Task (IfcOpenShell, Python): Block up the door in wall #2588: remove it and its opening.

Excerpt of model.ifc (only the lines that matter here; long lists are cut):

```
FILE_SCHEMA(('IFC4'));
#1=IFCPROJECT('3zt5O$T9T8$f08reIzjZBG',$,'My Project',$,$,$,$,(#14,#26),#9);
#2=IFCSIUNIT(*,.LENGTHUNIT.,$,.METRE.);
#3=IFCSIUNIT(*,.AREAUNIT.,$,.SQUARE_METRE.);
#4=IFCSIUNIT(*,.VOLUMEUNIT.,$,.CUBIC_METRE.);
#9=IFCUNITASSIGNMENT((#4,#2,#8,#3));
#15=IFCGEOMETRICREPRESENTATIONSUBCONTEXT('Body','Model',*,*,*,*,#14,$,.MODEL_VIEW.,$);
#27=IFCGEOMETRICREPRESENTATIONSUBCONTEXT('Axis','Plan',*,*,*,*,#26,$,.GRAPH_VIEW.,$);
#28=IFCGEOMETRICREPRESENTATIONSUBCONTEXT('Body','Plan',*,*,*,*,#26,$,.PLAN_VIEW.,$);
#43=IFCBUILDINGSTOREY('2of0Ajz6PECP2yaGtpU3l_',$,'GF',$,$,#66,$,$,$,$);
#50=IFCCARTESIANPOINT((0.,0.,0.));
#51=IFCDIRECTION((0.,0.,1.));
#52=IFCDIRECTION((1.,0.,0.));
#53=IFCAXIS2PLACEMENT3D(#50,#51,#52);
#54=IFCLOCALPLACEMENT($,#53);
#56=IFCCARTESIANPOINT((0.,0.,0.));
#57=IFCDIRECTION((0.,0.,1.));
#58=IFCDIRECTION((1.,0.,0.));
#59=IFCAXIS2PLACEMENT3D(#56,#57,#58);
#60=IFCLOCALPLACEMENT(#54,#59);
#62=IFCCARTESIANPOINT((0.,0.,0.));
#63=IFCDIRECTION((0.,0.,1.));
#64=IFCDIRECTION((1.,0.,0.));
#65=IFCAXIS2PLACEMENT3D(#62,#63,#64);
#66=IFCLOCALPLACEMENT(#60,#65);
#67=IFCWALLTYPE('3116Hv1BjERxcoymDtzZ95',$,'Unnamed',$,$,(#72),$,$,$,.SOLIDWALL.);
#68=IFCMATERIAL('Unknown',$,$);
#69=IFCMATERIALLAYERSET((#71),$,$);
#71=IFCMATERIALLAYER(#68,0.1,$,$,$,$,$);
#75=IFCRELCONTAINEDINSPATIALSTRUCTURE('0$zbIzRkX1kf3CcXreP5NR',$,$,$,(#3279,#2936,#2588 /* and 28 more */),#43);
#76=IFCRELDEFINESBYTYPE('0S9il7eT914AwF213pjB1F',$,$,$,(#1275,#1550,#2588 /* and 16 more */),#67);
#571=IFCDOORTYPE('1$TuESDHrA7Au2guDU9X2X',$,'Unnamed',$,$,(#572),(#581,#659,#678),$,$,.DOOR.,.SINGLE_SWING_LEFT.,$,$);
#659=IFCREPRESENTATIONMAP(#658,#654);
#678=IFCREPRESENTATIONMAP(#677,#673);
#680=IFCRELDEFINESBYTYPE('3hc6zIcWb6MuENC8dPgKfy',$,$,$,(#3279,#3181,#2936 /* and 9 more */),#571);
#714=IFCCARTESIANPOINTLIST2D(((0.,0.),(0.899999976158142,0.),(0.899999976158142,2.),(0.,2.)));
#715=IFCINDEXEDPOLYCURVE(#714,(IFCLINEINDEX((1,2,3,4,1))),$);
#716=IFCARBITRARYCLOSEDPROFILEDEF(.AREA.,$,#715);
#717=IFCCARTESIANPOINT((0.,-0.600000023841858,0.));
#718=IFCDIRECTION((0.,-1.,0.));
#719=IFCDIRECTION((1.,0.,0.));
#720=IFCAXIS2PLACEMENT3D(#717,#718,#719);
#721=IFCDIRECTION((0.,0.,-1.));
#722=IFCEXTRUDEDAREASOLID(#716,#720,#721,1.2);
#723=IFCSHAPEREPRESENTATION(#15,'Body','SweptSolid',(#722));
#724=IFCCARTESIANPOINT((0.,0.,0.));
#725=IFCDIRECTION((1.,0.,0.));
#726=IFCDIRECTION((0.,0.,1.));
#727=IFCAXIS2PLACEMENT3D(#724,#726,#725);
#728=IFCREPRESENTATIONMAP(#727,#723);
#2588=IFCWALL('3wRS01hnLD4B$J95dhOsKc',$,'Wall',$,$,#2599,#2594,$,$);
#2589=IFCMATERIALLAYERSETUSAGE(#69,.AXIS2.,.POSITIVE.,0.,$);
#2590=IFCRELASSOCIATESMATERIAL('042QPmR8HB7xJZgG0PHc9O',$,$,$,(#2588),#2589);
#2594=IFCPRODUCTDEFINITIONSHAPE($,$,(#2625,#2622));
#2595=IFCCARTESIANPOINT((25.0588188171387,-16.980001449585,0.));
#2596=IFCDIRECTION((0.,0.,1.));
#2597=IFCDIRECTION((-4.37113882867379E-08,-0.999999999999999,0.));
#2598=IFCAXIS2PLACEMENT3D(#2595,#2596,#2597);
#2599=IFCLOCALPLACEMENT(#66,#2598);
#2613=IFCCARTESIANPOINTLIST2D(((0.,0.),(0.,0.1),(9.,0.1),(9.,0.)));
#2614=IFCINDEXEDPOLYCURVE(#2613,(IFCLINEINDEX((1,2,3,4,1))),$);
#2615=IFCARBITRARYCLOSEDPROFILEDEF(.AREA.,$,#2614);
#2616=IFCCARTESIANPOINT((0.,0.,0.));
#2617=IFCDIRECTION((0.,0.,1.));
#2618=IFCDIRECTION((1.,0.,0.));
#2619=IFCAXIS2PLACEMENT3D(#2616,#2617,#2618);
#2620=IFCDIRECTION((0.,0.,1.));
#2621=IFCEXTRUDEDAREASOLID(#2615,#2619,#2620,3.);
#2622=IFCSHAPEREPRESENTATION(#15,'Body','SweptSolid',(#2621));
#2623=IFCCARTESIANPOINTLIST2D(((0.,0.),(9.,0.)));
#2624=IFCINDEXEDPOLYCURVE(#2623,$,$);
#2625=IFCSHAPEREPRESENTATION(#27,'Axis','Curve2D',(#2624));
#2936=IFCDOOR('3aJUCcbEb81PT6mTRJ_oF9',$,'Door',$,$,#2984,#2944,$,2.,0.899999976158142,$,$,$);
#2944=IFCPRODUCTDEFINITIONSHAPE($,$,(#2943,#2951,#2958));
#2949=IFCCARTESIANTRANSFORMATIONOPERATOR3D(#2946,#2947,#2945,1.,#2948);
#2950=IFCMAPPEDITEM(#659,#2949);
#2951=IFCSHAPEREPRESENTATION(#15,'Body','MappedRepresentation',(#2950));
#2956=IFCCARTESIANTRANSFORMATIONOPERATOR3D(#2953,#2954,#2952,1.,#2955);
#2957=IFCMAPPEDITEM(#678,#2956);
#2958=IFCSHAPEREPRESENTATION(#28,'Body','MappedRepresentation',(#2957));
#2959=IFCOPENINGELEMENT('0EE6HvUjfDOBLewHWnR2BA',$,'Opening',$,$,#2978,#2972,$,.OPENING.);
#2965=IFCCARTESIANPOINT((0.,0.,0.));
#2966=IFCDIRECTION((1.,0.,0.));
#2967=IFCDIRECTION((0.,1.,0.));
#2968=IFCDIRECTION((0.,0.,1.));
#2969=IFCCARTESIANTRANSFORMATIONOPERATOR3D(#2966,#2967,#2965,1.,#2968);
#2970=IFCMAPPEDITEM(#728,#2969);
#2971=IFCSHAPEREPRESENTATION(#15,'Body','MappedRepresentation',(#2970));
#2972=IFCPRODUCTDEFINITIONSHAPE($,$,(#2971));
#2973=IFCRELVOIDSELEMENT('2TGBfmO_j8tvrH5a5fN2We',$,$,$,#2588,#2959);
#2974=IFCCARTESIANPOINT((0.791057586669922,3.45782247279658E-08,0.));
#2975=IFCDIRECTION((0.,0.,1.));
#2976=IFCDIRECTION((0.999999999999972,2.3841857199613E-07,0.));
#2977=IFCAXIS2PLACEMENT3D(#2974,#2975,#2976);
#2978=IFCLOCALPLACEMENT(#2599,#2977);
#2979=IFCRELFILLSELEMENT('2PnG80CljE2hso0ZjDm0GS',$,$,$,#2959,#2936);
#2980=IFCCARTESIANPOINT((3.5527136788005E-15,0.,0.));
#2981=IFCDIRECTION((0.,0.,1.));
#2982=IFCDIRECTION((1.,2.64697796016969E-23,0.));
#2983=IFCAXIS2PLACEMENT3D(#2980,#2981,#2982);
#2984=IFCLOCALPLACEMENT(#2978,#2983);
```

```python
import ifcopenshell
import ifcopenshell.api.feature
import ifcopenshell.api.root
import ifcopenshell.geom
import ifcopenshell.util.shape

model = ifcopenshell.open("model.ifc")
settings = ifcopenshell.geom.settings()


def volume(element):
    """Net volume in cubic metres, openings subtracted."""
    shape = ifcopenshell.geom.create_shape(settings, element)
    return ifcopenshell.util.shape.get_volume(shape.geometry)


door = model.by_guid("3aJUCcbEb81PT6mTRJ_oF9")
opening = door.FillsVoids[0].RelatingOpeningElement
wall = opening.VoidsElements[0].RelatingBuildingElement
before = volume(wall)

ifcopenshell.api.root.remove_product(model, product=door)
ifcopenshell.api.feature.remove_feature(model, feature=opening)

after = volume(wall)

print(f"wall volume {before:.3f} -> {after:.3f} m3")

model.write("model_v2.ifc")
```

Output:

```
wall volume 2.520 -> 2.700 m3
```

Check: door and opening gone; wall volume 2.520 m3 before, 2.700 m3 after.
